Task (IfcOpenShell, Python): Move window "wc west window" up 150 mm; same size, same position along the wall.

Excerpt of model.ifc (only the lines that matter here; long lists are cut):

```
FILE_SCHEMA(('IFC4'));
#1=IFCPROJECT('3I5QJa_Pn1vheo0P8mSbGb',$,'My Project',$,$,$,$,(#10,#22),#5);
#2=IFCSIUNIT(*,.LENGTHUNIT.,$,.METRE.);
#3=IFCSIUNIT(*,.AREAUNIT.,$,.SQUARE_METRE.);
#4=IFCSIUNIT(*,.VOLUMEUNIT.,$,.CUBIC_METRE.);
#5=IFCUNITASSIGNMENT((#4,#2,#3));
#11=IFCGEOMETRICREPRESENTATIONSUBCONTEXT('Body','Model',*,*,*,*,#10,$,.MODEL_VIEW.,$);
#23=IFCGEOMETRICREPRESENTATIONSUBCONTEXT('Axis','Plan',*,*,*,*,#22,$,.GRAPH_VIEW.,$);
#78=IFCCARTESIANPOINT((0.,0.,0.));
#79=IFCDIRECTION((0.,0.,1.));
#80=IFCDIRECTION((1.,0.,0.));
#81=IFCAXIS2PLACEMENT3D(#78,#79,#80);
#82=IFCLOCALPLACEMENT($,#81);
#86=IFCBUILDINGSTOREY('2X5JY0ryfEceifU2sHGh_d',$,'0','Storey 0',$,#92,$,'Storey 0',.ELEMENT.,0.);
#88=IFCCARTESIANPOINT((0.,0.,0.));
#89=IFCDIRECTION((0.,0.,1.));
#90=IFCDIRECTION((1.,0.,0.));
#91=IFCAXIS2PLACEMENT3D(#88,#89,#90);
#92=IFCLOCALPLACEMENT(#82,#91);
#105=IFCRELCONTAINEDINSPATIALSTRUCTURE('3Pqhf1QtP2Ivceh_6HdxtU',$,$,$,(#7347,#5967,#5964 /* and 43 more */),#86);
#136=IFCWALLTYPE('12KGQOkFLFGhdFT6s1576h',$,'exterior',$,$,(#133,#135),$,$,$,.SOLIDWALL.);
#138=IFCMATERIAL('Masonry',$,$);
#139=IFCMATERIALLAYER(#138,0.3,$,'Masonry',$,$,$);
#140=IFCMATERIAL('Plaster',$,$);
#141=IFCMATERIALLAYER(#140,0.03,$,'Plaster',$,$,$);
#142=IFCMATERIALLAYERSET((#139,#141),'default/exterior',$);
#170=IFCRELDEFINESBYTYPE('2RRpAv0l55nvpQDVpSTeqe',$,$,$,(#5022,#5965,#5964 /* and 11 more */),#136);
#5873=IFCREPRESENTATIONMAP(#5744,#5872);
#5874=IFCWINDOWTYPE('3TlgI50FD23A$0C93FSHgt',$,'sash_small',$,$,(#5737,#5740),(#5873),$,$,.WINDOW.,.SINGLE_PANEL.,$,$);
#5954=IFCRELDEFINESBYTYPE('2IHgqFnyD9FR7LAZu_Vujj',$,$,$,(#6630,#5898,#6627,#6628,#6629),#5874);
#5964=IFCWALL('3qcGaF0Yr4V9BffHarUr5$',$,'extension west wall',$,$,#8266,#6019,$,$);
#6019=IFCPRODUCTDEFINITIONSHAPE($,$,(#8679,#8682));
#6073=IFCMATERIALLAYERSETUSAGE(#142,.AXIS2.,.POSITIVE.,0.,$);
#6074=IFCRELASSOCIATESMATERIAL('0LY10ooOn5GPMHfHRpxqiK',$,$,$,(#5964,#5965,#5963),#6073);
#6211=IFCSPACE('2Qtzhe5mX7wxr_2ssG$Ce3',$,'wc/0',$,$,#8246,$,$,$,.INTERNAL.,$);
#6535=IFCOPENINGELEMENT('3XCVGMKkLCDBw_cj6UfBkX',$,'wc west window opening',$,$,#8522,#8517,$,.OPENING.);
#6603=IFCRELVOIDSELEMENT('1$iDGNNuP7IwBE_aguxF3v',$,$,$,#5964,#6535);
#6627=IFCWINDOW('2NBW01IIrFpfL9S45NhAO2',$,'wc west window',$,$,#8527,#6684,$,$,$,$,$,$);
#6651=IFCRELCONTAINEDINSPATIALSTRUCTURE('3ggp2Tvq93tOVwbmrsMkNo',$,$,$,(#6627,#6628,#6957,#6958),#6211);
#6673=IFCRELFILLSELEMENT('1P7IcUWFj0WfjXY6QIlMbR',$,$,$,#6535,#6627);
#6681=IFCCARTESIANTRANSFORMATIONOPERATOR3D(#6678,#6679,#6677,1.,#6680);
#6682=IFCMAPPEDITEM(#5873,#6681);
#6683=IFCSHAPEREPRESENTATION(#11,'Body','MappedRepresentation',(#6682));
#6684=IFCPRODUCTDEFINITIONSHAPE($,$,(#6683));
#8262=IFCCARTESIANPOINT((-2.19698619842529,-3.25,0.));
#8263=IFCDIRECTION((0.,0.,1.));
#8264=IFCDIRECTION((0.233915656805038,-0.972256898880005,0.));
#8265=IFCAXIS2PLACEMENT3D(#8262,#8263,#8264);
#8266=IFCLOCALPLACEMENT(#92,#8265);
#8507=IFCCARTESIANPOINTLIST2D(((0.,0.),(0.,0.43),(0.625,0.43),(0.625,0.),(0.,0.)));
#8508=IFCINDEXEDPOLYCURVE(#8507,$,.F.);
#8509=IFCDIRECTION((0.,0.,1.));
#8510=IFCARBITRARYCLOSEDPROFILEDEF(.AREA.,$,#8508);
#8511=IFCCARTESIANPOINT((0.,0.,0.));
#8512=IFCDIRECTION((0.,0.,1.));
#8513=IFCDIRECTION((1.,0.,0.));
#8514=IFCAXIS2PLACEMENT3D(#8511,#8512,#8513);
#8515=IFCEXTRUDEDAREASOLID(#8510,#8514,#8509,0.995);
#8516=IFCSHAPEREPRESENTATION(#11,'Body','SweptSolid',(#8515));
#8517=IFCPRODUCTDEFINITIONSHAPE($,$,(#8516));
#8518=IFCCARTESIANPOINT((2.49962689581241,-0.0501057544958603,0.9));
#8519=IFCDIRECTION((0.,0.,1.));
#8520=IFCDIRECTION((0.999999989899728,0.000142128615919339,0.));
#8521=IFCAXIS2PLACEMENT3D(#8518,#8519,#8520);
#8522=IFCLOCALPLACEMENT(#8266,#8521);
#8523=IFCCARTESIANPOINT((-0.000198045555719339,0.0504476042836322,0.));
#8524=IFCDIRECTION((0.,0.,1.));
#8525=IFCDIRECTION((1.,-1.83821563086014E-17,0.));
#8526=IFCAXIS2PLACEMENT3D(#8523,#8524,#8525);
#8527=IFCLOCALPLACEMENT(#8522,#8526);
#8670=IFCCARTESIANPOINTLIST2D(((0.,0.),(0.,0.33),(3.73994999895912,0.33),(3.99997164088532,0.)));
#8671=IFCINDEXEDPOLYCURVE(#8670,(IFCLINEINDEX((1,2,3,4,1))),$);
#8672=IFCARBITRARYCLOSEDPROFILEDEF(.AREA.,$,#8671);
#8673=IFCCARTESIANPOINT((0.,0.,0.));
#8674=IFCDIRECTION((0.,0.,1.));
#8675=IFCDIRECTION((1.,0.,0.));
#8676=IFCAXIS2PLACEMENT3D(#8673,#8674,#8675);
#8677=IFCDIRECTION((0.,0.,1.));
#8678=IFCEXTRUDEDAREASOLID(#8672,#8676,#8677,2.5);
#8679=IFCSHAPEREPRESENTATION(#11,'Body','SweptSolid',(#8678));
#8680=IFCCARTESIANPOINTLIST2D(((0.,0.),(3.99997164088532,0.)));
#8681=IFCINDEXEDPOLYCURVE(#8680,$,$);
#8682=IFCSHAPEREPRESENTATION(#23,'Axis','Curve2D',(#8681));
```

```python
import numpy as np
import ifcopenshell
import ifcopenshell.api.geometry
import ifcopenshell.util.placement
import ifcopenshell.util.unit

model = ifcopenshell.open("model.ifc")
unit_scale = ifcopenshell.util.unit.calculate_unit_scale(model)

window = model.by_guid("2NBW01IIrFpfL9S45NhAO2")
opening = window.FillsVoids[0].RelatingOpeningElement
dz = 0.15 / unit_scale

shift = np.array([0.0, 0.0, dz])
# The window is placed relative to its opening, so it follows when the opening moves.
matrix = ifcopenshell.util.placement.get_local_placement(opening.ObjectPlacement)
matrix[:3, 3] += shift
ifcopenshell.api.geometry.edit_object_placement(
    model, product=opening, matrix=matrix, is_si=False, should_transform_children=True
)

print(f"moved by {dz * unit_scale:+.3f} m")

model.write("model-out.ifc")
```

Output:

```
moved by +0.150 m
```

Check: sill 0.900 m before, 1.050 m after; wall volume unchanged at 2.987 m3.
